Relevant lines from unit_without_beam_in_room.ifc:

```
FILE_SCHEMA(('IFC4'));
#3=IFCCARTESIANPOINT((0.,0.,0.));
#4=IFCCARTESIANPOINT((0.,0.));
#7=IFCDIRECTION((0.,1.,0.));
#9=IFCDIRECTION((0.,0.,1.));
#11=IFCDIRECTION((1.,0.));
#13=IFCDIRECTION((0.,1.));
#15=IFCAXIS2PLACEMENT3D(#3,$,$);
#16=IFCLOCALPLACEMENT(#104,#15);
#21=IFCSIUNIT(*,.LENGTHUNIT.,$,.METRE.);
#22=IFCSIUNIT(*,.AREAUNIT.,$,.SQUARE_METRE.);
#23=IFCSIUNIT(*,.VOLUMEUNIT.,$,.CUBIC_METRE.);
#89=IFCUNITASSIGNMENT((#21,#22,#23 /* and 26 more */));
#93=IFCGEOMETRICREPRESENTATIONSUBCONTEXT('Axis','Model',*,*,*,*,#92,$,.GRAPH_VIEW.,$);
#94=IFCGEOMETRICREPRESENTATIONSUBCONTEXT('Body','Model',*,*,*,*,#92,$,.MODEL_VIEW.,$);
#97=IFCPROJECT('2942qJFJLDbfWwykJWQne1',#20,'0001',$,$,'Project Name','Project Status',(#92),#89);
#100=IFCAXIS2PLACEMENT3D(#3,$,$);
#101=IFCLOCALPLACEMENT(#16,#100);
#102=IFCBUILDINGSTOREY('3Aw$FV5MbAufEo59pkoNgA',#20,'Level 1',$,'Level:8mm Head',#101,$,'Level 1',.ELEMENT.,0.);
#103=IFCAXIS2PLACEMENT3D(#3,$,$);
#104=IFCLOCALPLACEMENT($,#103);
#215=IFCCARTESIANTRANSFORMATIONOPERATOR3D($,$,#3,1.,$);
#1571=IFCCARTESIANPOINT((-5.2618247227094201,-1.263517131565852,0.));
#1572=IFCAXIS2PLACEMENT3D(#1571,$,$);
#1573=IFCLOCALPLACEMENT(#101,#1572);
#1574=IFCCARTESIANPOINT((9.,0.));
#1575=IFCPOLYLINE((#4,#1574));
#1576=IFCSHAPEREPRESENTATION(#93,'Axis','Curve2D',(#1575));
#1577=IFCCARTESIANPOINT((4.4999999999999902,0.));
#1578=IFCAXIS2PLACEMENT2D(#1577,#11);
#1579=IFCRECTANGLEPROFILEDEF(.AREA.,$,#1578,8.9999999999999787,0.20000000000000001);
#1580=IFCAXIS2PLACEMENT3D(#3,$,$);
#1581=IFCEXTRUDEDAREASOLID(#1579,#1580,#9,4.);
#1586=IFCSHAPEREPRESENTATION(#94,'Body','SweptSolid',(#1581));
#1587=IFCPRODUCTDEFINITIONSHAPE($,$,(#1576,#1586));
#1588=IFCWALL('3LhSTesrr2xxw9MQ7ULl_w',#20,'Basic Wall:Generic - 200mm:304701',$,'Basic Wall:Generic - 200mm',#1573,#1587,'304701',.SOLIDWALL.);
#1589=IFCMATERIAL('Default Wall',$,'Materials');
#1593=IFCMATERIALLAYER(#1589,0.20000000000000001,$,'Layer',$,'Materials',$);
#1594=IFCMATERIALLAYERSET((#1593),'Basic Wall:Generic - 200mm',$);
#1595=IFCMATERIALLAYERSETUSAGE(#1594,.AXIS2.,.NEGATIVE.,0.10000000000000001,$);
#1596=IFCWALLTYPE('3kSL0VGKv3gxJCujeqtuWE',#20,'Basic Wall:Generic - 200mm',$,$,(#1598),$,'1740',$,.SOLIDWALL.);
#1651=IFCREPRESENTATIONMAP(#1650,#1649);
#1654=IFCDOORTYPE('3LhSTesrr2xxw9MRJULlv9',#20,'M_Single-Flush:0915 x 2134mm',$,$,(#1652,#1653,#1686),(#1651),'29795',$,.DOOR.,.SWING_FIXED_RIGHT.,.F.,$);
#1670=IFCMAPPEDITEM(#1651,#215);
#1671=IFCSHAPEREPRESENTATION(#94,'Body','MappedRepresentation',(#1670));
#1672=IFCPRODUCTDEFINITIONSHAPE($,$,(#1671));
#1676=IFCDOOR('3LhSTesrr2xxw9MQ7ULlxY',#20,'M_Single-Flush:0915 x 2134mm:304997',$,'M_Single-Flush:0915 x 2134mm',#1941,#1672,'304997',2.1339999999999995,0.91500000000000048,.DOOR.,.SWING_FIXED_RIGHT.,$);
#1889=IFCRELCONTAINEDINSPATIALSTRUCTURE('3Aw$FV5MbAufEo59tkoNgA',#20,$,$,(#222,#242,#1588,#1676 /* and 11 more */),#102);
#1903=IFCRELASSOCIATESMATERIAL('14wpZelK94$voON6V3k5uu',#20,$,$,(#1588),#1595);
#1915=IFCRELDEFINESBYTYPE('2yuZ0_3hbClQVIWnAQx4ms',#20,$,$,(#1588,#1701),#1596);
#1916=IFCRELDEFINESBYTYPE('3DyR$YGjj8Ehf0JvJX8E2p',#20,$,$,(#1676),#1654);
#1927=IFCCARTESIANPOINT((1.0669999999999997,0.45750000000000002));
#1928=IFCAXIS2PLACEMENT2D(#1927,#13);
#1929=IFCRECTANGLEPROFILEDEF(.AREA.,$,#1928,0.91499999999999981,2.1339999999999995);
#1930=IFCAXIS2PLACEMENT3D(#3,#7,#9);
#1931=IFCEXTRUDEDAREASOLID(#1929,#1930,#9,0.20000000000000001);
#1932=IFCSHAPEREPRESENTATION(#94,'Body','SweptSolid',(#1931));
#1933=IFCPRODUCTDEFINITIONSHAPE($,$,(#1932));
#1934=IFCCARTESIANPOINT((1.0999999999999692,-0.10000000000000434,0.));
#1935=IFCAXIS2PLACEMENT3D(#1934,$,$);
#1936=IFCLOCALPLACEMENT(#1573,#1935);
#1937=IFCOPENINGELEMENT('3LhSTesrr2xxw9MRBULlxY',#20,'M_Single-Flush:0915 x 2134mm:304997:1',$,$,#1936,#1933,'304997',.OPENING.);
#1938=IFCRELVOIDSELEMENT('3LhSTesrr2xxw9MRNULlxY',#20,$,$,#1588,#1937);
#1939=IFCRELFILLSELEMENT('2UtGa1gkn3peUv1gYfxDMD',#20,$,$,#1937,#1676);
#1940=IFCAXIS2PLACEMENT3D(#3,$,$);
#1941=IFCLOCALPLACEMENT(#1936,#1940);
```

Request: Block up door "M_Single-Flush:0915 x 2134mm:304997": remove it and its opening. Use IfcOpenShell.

```python
import ifcopenshell
import ifcopenshell.api.feature
import ifcopenshell.api.root
import ifcopenshell.geom
import ifcopenshell.util.shape

model = ifcopenshell.open("unit_without_beam_in_room.ifc")
settings = ifcopenshell.geom.settings()


def volume(element):
    """Net volume in cubic metres, openings subtracted."""
    shape = ifcopenshell.geom.create_shape(settings, element)
    return ifcopenshell.util.shape.get_volume(shape.geometry)


door = model.by_id(1676)
opening = door.FillsVoids[0].RelatingOpeningElement
wall = opening.VoidsElements[0].RelatingBuildingElement
before = volume(wall)

ifcopenshell.api.root.remove_product(model, product=door)
ifcopenshell.api.feature.remove_feature(model, feature=opening)

after = volume(wall)

print(f"wall volume {before:.3f} -> {after:.3f} m3")

model.write("unit_without_beam_in_room_rev.ifc")
```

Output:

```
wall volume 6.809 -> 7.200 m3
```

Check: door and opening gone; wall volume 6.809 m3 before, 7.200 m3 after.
